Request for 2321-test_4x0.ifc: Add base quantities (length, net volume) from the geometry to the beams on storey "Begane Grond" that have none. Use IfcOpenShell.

First a look at what the model holds.

```python
import ifcopenshell
import ifcopenshell.util.element
import ifcopenshell.util.unit

model = ifcopenshell.open("2321-test_4x0.ifc")
print(model.schema)
for unit_type in ("LENGTHUNIT", "AREAUNIT", "VOLUMEUNIT"):
    print(unit_type, ifcopenshell.util.unit.calculate_unit_scale(model, unit_type))
storey = next(s for s in model.by_type("IfcBuildingStorey") if s.Name == "Begane Grond")
beams = [e for e in ifcopenshell.util.element.get_decomposition(storey) if e.is_a("IfcBeam")]
for e in sorted(beams, key=lambda e: e.id()):
    print(e.id(), e.is_a(), e.Name, list(ifcopenshell.util.element.get_psets(e, qtos_only=True)), sep=" | ")
```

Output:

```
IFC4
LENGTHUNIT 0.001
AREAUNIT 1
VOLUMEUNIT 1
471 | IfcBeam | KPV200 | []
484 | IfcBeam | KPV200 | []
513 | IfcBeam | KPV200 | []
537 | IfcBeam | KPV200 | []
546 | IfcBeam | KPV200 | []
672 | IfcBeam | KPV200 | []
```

```python
import ifcopenshell
import ifcopenshell.api.pset
import ifcopenshell.geom
import ifcopenshell.util.element
import ifcopenshell.util.shape
import ifcopenshell.util.unit

model = ifcopenshell.open("2321-test_4x0.ifc")
unit_scale = ifcopenshell.util.unit.calculate_unit_scale(model)
volume_scale = ifcopenshell.util.unit.calculate_unit_scale(model, "VOLUMEUNIT")
settings = ifcopenshell.geom.settings()

storey = next(s for s in model.by_type("IfcBuildingStorey") if s.Name == "Begane Grond")
beams = [e for e in ifcopenshell.util.element.get_decomposition(storey) if e.is_a("IfcBeam")]

for e in sorted(beams, key=lambda e: e.id()):
    if ifcopenshell.util.element.get_psets(e, qtos_only=True, should_inherit=False):
        continue
    # Geometry comes back in metres, in the element's own axes.
    shape = ifcopenshell.geom.create_shape(settings, e)
    values = {
        "Length": ifcopenshell.util.shape.get_max_xyz(shape.geometry) / unit_scale,
        "NetVolume": ifcopenshell.util.shape.get_volume(shape.geometry) / volume_scale,
    }
    qto = ifcopenshell.api.pset.add_qto(model, product=e, name="Qto_BeamBaseQuantities")
    ifcopenshell.api.pset.edit_qto(model, qto=qto, properties=values)
    print(e.id(), {k: round(v, 3) for k, v in values.items()})

model.write("2321-test_4x0_updated.ifc")
```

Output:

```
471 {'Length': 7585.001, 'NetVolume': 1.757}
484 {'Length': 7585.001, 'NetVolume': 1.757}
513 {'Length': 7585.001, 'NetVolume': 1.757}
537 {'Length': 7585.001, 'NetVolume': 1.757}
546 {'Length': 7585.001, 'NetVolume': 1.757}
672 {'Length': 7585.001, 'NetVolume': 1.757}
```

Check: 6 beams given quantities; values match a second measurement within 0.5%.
